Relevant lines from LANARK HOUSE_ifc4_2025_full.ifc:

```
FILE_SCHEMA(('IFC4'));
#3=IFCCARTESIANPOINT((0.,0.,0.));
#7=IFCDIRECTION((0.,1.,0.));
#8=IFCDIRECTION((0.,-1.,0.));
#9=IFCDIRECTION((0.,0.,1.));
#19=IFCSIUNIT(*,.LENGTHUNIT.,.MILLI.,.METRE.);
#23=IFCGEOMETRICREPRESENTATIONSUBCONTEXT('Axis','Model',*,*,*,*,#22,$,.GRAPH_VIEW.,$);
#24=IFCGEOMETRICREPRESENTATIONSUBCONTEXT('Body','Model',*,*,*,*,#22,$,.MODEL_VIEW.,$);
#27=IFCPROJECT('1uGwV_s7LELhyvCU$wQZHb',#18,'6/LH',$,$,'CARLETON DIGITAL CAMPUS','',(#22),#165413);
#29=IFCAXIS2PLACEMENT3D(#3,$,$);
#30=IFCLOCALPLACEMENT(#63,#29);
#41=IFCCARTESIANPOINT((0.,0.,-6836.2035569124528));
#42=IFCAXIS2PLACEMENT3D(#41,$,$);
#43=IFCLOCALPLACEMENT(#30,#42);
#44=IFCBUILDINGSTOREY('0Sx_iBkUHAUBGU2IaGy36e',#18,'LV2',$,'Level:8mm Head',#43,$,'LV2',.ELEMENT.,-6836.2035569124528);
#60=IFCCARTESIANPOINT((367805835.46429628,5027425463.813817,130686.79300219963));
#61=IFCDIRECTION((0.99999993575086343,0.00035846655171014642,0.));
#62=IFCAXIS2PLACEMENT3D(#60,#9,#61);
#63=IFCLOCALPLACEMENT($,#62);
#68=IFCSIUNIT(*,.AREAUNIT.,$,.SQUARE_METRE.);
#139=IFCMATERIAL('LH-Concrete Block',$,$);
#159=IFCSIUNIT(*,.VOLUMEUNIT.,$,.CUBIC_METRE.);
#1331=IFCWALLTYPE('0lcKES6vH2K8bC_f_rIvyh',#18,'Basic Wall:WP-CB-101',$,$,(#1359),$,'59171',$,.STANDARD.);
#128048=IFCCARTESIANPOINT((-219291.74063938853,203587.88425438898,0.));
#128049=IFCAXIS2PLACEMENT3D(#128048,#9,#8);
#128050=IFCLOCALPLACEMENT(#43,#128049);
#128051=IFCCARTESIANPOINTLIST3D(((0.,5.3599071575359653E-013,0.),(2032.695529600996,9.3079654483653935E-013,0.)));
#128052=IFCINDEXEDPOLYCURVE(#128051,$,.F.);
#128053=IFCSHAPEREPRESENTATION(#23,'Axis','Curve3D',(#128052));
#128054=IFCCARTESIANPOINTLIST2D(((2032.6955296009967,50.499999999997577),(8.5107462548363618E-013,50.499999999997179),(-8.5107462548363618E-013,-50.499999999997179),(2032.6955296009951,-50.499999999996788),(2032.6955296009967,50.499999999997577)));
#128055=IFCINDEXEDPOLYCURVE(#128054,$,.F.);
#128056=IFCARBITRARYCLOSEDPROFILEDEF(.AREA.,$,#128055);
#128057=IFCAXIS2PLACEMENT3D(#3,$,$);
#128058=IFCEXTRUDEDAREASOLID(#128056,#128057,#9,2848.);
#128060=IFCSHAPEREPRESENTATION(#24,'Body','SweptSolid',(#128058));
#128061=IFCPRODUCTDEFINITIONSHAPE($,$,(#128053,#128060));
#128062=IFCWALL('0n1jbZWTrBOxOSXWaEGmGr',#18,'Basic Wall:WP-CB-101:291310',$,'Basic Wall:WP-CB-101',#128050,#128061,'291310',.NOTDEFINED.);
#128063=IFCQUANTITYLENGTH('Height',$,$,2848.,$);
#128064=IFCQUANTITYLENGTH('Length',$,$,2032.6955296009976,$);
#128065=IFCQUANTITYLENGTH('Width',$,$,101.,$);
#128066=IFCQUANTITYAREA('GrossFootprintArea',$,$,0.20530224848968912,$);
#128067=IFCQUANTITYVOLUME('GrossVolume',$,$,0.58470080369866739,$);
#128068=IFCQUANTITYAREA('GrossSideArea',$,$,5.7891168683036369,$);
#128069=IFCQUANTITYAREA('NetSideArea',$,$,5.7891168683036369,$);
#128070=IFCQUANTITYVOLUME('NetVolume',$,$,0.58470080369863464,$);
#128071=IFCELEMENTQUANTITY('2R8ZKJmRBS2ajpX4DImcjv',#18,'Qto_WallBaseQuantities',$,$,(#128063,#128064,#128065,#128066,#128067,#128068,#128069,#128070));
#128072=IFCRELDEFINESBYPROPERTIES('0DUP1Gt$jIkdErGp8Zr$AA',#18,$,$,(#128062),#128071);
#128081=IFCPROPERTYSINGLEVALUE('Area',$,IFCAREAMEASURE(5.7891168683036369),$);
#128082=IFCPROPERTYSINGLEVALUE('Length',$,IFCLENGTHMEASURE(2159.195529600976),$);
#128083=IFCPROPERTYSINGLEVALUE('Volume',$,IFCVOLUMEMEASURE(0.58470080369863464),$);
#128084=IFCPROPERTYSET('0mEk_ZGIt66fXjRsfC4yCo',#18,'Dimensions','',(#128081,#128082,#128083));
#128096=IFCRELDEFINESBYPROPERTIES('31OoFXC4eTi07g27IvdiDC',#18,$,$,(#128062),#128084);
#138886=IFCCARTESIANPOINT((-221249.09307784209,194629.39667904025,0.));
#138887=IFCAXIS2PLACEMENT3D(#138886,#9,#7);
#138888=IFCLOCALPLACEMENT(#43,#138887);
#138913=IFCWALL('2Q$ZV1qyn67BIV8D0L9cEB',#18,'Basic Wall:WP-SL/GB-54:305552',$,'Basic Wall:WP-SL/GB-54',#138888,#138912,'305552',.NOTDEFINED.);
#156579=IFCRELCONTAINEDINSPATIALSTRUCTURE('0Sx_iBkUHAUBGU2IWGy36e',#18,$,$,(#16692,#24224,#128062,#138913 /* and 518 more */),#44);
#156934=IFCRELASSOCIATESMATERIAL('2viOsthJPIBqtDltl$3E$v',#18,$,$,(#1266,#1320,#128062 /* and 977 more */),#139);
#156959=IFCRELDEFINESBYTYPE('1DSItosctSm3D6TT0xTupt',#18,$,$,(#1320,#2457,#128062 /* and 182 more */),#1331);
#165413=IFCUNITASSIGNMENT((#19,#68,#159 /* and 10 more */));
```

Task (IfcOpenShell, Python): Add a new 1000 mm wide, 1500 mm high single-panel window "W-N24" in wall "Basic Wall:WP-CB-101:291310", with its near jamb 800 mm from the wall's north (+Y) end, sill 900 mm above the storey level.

```python
import numpy as np
import ifcopenshell
import ifcopenshell.api.feature
import ifcopenshell.api.geometry
import ifcopenshell.api.pset
import ifcopenshell.api.root
import ifcopenshell.api.spatial
import ifcopenshell.geom
import ifcopenshell.util.element
import ifcopenshell.util.placement
import ifcopenshell.util.representation
import ifcopenshell.util.shape
import ifcopenshell.util.unit

model = ifcopenshell.open("LANARK HOUSE_ifc4_2025_full.ifc")
unit_scale = ifcopenshell.util.unit.calculate_unit_scale(model)
area_scale = ifcopenshell.util.unit.calculate_unit_scale(model, "AREAUNIT")
volume_scale = ifcopenshell.util.unit.calculate_unit_scale(model, "VOLUMEUNIT")
settings = ifcopenshell.geom.settings()


def volume(element):
    """Net volume in cubic metres, openings subtracted."""
    shape = ifcopenshell.geom.create_shape(settings, element)
    return ifcopenshell.util.shape.get_volume(shape.geometry)


wall = model.by_guid("0n1jbZWTrBOxOSXWaEGmGr")
storey = ifcopenshell.util.element.get_container(wall, ifc_class="IfcBuildingStorey")
context = ifcopenshell.util.representation.get_context(model, "Model", "Body", "MODEL_VIEW")
before = volume(wall)

width, height, from_end, sill = 1, 1.5, 0.8, 0.9  # metres

# The wall runs along its own X axis, and the end named is its -X end.
wall_shape = ifcopenshell.geom.create_shape(settings, wall)
x, y, z = ifcopenshell.util.shape.get_vertices(wall_shape.geometry).T
start = x.min() + from_end
face, thickness = float(y.min()), float(y.max() - y.min())
wall_matrix = ifcopenshell.util.placement.get_local_placement(wall.ObjectPlacement)
level = ifcopenshell.util.placement.get_local_placement(storey.ObjectPlacement)[2, 3]


def in_wall(x, y):
    """Placement at x, y metres in the wall's axes, at sill height."""
    matrix = wall_matrix.copy()
    matrix[:, 3] = wall_matrix @ np.array([x / unit_scale, y / unit_scale, 0.0, 1.0])
    matrix[2, 3] = level + sill / unit_scale
    return matrix


# Opening: a box that overshoots both wall faces by 50 mm.
opening = ifcopenshell.api.root.create_entity(model, ifc_class="IfcOpeningElement", predefined_type="OPENING")
box = ifcopenshell.api.geometry.add_wall_representation(
    model, context=context, length=width, height=height, thickness=thickness + 0.1
)
ifcopenshell.api.geometry.assign_representation(model, product=opening, representation=box)
ifcopenshell.api.geometry.edit_object_placement(model, product=opening, matrix=in_wall(start, face - 0.05), is_si=False)
ifcopenshell.api.feature.add_feature(model, feature=opening, element=wall)

window = ifcopenshell.api.root.create_entity(model, ifc_class="IfcWindow", name="W-N24", predefined_type="WINDOW")
window.OverallWidth, window.OverallHeight = width / unit_scale, height / unit_scale
window.PartitioningType = "SINGLE_PANEL"
body = ifcopenshell.api.geometry.add_window_representation(
    model,
    context=context,
    overall_width=window.OverallWidth,
    overall_height=window.OverallHeight,
    partition_type="SINGLE_PANEL",
)
ifcopenshell.api.geometry.assign_representation(model, product=window, representation=body)
ifcopenshell.api.spatial.assign_container(model, products=[window], relating_structure=storey)
ifcopenshell.api.feature.add_filling(model, opening=opening, element=window)

# Centre the window in the wall's thickness.
ifcopenshell.api.geometry.edit_object_placement(model, product=window, matrix=in_wall(start, face), is_si=False)
window_shape = ifcopenshell.geom.create_shape(settings, window)
depth = ifcopenshell.util.shape.get_vertices(window_shape.geometry)[:, 1]
offset = face + thickness / 2 - (depth.min() + depth.max()) / 2
ifcopenshell.api.geometry.edit_object_placement(model, product=window, matrix=in_wall(start, offset), is_si=False)

after = volume(wall)

# Update the wall's stored quantities.
qto = model.by_id(ifcopenshell.util.element.get_pset(wall, "Qto_WallBaseQuantities", should_inherit=False)["id"])
ifcopenshell.api.pset.edit_qto(model, qto=qto, properties={
    "NetSideArea": after / thickness / area_scale,
    "NetVolume": after / volume_scale,
})
pset = model.by_id(ifcopenshell.util.element.get_pset(wall, "Dimensions", should_inherit=False)["id"])
ifcopenshell.api.pset.edit_pset(model, pset=pset, properties={
    "Area": model.create_entity("IfcAreaMeasure", after / thickness / area_scale),
    "Volume": model.create_entity("IfcVolumeMeasure", after / volume_scale),
})

print(f"wall volume {before:.3f} -> {after:.3f} m3")

model.write("LANARK HOUSE_ifc4_2025_full_v2.ifc")
```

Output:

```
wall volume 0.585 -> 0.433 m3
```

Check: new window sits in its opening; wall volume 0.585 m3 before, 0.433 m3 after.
